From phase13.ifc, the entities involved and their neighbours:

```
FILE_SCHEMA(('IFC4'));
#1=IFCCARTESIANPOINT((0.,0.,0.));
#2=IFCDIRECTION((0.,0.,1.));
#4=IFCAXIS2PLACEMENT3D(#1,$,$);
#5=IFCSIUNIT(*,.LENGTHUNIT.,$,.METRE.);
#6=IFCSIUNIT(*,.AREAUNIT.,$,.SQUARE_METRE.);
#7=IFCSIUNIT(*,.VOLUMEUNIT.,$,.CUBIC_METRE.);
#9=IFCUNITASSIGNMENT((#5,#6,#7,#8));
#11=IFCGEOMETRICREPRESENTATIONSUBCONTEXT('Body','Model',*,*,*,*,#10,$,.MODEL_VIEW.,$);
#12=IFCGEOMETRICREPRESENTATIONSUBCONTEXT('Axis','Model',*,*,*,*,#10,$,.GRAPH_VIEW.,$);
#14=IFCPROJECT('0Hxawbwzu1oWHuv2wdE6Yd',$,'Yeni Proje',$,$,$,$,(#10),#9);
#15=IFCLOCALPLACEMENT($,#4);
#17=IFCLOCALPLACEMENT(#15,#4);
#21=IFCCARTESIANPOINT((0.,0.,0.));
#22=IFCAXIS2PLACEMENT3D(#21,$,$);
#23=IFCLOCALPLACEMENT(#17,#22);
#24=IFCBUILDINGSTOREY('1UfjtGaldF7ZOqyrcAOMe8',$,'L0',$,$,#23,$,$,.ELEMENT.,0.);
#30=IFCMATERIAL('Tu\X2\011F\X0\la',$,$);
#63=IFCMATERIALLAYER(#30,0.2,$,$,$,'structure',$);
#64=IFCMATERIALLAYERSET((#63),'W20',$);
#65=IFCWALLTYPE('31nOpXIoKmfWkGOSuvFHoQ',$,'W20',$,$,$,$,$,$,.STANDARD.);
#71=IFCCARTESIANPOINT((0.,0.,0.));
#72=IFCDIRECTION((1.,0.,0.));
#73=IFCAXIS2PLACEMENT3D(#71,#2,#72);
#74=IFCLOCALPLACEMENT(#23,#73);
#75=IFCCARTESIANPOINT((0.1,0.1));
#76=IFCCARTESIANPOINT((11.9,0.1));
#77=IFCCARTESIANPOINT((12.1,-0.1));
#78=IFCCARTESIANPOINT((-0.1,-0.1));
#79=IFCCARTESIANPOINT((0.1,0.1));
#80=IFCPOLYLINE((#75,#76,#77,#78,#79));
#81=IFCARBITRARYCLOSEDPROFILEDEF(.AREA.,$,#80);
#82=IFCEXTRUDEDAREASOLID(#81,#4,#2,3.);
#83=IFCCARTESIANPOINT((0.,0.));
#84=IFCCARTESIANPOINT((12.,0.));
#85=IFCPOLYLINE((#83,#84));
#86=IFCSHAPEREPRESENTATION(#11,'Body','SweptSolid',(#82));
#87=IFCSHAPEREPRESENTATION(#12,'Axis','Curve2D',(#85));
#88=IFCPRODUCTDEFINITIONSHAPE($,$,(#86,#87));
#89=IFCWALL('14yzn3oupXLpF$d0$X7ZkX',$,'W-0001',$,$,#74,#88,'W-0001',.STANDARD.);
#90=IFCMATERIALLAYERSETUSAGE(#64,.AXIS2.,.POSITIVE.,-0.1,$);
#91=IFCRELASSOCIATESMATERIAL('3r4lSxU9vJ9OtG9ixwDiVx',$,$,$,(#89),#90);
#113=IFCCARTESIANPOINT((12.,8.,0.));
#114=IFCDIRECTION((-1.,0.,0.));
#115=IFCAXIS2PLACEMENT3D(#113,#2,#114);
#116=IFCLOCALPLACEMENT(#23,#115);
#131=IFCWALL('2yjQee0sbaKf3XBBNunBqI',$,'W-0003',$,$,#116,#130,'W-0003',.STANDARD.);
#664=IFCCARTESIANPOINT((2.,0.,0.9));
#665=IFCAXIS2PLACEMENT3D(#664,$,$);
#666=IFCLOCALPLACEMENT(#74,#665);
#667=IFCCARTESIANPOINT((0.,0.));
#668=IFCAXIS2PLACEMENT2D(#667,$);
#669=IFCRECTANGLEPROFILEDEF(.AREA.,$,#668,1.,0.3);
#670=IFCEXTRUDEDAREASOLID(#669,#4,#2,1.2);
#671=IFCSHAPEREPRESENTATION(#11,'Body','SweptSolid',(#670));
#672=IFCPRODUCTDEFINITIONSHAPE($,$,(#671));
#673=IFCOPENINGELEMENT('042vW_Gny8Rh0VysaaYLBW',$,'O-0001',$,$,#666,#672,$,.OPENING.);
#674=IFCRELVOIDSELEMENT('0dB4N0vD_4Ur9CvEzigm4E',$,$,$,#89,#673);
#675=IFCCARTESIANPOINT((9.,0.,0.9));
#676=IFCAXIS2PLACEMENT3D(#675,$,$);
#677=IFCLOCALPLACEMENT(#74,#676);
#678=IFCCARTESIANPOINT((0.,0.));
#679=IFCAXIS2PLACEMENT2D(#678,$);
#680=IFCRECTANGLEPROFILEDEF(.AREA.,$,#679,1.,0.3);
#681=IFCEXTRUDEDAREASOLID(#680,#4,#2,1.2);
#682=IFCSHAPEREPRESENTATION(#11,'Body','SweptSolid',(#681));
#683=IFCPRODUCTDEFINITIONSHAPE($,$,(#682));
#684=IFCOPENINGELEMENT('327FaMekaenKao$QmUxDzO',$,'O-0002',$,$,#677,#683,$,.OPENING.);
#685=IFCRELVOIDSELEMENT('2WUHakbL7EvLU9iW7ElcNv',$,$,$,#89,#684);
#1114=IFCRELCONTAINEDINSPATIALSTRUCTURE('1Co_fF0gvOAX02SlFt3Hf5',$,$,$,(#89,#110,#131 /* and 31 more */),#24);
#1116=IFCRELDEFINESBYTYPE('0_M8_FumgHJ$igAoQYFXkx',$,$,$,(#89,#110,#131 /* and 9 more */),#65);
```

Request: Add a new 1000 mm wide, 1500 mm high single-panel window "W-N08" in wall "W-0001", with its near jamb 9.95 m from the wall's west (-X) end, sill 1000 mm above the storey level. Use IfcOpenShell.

```python
import numpy as np
import ifcopenshell
import ifcopenshell.api.feature
import ifcopenshell.api.geometry
import ifcopenshell.api.root
import ifcopenshell.api.spatial
import ifcopenshell.geom
import ifcopenshell.util.element
import ifcopenshell.util.placement
import ifcopenshell.util.representation
import ifcopenshell.util.shape
import ifcopenshell.util.unit

model = ifcopenshell.open("phase13.ifc")
unit_scale = ifcopenshell.util.unit.calculate_unit_scale(model)
settings = ifcopenshell.geom.settings()


def volume(element):
    """Net volume in cubic metres, openings subtracted."""
    shape = ifcopenshell.geom.create_shape(settings, element)
    return ifcopenshell.util.shape.get_volume(shape.geometry)


wall = model.by_guid("14yzn3oupXLpF$d0$X7ZkX")
storey = ifcopenshell.util.element.get_container(wall, ifc_class="IfcBuildingStorey")
context = ifcopenshell.util.representation.get_context(model, "Model", "Body", "MODEL_VIEW")
before = volume(wall)

width, height, from_end, sill = 1, 1.5, 9.95, 1  # metres

# The wall runs along its own X axis, and the end named is its -X end.
wall_shape = ifcopenshell.geom.create_shape(settings, wall)
x, y, z = ifcopenshell.util.shape.get_vertices(wall_shape.geometry).T
start = x.min() + from_end
face, thickness = float(y.min()), float(y.max() - y.min())
wall_matrix = ifcopenshell.util.placement.get_local_placement(wall.ObjectPlacement)
level = ifcopenshell.util.placement.get_local_placement(storey.ObjectPlacement)[2, 3]


def in_wall(x, y):
    """Placement at x, y metres in the wall's axes, at sill height."""
    matrix = wall_matrix.copy()
    matrix[:, 3] = wall_matrix @ np.array([x / unit_scale, y / unit_scale, 0.0, 1.0])
    matrix[2, 3] = level + sill / unit_scale
    return matrix


# Opening: a box that overshoots both wall faces by 50 mm.
opening = ifcopenshell.api.root.create_entity(model, ifc_class="IfcOpeningElement", predefined_type="OPENING")
box = ifcopenshell.api.geometry.add_wall_representation(
    model, context=context, length=width, height=height, thickness=thickness + 0.1
)
ifcopenshell.api.geometry.assign_representation(model, product=opening, representation=box)
ifcopenshell.api.geometry.edit_object_placement(model, product=opening, matrix=in_wall(start, face - 0.05), is_si=False)
ifcopenshell.api.feature.add_feature(model, feature=opening, element=wall)

window = ifcopenshell.api.root.create_entity(model, ifc_class="IfcWindow", name="W-N08", predefined_type="WINDOW")
window.OverallWidth, window.OverallHeight = width / unit_scale, height / unit_scale
window.PartitioningType = "SINGLE_PANEL"
body = ifcopenshell.api.geometry.add_window_representation(
    model,
    context=context,
    overall_width=window.OverallWidth,
    overall_height=window.OverallHeight,
    partition_type="SINGLE_PANEL",
)
ifcopenshell.api.geometry.assign_representation(model, product=window, representation=body)
ifcopenshell.api.spatial.assign_container(model, products=[window], relating_structure=storey)
ifcopenshell.api.feature.add_filling(model, opening=opening, element=window)

# Centre the window in the wall's thickness.
ifcopenshell.api.geometry.edit_object_placement(model, product=window, matrix=in_wall(start, face), is_si=False)
window_shape = ifcopenshell.geom.create_shape(settings, window)
depth = ifcopenshell.util.shape.get_vertices(window_shape.geometry)[:, 1]
offset = face + thickness / 2 - (depth.min() + depth.max()) / 2
ifcopenshell.api.geometry.edit_object_placement(model, product=window, matrix=in_wall(start, offset), is_si=False)

after = volume(wall)

print(f"wall volume {before:.3f} -> {after:.3f} m3")

model.write("phase13_rev.ifc")
```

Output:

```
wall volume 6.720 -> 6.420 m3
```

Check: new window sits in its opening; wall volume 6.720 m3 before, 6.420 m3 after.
